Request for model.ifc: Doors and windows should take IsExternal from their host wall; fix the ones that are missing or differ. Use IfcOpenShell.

First a look at what the model holds.

```python
import ifcopenshell
import ifcopenshell.util.element

model = ifcopenshell.open("model.ifc")
print(model.schema)
seen = {}
for e in model.by_type("IfcDoor") + model.by_type("IfcWindow"):
    if not e.FillsVoids:
        continue
    host = e.FillsVoids[0].RelatingOpeningElement.VoidsElements[0].RelatingBuildingElement
    own = ifcopenshell.util.element.get_pset(e, f"Pset_{e.is_a()[3:].removesuffix('StandardCase')}Common", "IsExternal")
    wall = ifcopenshell.util.element.get_pset(host, "Pset_WallCommon", "IsExternal")
    seen[e.is_a(), own, wall] = seen.get((e.is_a(), own, wall), 0) + 1
for (cls, own, wall), count in sorted(seen.items(), key=str):
    print(count, cls, "IsExternal:", own, "| host wall:", wall)
```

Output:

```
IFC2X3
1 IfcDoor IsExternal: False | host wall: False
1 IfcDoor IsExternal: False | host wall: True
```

```python
import ifcopenshell
import ifcopenshell.api.pset
import ifcopenshell.util.element

model = ifcopenshell.open("model.ifc")

count = 0
for ifc_class, pset_name in (("IfcDoor", "Pset_DoorCommon"), ("IfcWindow", "Pset_WindowCommon")):
    for e in model.by_type(ifc_class):
        if not e.FillsVoids:
            continue
        host = e.FillsVoids[0].RelatingOpeningElement.VoidsElements[0].RelatingBuildingElement
        external = ifcopenshell.util.element.get_pset(host, "Pset_WallCommon", "IsExternal")
        if external is None or ifcopenshell.util.element.get_pset(e, pset_name, "IsExternal") == external:
            continue
        pset = ifcopenshell.api.pset.add_pset(model, product=e, name=pset_name)
        ifcopenshell.api.pset.edit_pset(model, pset=pset, properties={"IsExternal": external})
        count += 1

print(count, "updated")

model.write("model_v2.ifc")
```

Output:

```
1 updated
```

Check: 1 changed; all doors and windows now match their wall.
